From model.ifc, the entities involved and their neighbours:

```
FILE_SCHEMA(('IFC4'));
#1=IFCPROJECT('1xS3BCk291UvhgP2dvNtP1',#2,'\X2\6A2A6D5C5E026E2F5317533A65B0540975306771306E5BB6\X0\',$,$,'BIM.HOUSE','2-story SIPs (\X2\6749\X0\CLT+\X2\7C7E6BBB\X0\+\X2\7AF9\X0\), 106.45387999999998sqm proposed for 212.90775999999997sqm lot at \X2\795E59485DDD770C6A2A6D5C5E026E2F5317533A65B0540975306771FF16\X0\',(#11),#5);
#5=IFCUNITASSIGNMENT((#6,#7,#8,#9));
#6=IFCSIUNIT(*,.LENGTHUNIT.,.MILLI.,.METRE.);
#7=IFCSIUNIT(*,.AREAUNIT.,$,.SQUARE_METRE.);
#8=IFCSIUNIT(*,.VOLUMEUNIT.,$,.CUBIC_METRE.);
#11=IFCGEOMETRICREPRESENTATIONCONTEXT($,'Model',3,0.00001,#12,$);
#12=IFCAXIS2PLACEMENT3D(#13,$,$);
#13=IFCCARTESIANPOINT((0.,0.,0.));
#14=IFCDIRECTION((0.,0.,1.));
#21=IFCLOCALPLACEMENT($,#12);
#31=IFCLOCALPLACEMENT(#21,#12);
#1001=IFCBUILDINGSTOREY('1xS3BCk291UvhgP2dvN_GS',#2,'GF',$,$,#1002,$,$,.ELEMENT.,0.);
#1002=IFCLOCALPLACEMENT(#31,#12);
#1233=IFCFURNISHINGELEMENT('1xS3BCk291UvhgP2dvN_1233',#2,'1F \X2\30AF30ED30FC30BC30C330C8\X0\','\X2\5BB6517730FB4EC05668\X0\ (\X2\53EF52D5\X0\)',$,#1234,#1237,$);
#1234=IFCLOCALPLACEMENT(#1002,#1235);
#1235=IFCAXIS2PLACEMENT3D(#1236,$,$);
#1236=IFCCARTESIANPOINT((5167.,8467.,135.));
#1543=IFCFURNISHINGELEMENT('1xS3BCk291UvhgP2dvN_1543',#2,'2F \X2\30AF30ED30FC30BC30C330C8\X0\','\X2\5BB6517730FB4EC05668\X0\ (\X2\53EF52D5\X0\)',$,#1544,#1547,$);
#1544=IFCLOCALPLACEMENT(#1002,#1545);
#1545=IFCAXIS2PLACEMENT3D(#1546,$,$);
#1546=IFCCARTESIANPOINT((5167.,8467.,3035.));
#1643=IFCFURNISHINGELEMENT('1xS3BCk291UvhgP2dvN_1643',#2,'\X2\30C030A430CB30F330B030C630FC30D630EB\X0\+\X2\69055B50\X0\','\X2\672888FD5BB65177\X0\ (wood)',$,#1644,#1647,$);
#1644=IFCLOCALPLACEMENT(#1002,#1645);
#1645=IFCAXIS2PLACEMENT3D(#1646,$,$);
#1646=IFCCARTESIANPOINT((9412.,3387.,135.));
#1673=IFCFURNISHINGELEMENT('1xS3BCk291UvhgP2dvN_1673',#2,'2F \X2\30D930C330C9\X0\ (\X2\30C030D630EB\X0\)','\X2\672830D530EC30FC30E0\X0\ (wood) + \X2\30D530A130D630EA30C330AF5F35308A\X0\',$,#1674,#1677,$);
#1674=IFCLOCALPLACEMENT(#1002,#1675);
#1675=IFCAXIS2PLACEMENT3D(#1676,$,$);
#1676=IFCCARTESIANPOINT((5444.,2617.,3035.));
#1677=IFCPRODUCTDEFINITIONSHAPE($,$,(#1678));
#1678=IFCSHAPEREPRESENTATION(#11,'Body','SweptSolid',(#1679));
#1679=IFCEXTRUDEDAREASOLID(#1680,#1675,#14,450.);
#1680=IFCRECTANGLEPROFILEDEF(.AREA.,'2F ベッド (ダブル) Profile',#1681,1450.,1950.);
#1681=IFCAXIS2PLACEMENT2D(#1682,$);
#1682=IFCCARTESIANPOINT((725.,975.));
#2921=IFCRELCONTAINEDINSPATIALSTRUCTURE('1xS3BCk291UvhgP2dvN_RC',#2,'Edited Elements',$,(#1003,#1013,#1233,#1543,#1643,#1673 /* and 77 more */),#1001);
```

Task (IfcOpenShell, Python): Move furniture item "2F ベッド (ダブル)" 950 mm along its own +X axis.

```python
import ifcopenshell
import ifcopenshell.api.geometry
import ifcopenshell.util.placement
import ifcopenshell.util.unit

model = ifcopenshell.open("model.ifc")
unit_scale = ifcopenshell.util.unit.calculate_unit_scale(model)

item = model.by_guid("1xS3BCk291UvhgP2dvN_1673")
matrix = ifcopenshell.util.placement.get_local_placement(item.ObjectPlacement)
matrix[:3, 3] += matrix[:3, 0] * 0.95 / unit_scale
ifcopenshell.api.geometry.edit_object_placement(model, product=item, matrix=matrix, is_si=False)

print(ifcopenshell.util.placement.get_local_placement(item.ObjectPlacement).round(3) + 0.0)

model.write("model_updated.ifc")
```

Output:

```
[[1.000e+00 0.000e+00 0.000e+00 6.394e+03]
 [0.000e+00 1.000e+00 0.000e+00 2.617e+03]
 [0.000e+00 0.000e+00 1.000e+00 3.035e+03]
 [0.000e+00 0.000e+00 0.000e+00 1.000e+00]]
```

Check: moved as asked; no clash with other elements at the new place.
